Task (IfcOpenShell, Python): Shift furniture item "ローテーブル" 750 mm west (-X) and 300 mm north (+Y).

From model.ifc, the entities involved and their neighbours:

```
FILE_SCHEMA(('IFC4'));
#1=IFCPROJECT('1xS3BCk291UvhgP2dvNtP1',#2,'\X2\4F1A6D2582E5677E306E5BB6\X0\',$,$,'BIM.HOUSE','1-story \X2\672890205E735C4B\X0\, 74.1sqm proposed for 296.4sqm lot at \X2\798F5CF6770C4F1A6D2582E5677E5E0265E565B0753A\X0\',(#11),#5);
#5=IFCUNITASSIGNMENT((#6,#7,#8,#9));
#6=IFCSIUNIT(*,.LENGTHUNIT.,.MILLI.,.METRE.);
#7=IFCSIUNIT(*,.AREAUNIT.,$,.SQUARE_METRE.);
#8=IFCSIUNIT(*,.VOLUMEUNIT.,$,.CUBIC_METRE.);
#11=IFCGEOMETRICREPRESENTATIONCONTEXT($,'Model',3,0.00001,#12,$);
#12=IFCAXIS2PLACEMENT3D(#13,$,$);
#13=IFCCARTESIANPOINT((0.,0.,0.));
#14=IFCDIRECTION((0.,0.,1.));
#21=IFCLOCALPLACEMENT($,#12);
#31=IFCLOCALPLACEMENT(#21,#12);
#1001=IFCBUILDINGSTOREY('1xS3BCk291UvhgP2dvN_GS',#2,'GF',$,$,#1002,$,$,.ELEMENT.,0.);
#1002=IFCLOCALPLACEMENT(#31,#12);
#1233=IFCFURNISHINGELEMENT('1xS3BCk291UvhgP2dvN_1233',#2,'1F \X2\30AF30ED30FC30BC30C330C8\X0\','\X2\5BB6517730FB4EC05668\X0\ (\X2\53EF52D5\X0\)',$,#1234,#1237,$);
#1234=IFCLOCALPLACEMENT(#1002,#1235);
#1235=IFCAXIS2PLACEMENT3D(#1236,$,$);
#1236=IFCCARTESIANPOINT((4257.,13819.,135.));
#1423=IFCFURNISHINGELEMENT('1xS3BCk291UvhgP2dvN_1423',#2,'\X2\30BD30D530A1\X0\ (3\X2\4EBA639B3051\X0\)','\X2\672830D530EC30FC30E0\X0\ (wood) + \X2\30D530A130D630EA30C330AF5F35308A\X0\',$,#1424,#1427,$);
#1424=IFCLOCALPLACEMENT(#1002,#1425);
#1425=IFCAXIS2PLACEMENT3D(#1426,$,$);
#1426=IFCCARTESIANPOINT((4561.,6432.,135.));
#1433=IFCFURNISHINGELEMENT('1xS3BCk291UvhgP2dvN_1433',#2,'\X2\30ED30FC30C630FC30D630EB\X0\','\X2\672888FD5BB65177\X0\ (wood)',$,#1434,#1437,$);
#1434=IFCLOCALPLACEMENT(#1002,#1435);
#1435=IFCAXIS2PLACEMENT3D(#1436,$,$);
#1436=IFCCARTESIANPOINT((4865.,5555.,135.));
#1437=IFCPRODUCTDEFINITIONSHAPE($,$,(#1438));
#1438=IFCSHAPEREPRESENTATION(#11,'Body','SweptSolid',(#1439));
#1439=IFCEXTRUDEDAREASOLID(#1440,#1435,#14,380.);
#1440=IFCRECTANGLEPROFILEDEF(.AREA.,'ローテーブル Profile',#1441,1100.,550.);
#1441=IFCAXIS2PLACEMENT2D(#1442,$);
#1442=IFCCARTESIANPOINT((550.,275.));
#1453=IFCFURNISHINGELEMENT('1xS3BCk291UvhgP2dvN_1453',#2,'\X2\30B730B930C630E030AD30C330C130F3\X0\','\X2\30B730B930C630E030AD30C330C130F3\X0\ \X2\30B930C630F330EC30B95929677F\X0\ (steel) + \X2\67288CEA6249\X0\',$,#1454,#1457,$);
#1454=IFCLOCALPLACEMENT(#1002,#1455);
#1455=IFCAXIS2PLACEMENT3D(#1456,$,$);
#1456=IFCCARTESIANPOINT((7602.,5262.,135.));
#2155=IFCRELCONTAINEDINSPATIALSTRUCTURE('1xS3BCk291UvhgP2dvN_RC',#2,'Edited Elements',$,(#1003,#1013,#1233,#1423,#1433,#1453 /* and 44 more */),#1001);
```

```python
import ifcopenshell
import ifcopenshell.api.geometry
import ifcopenshell.util.placement
import ifcopenshell.util.unit

model = ifcopenshell.open("model.ifc")
unit_scale = ifcopenshell.util.unit.calculate_unit_scale(model)

item = model.by_guid("1xS3BCk291UvhgP2dvN_1433")
matrix = ifcopenshell.util.placement.get_local_placement(item.ObjectPlacement)
matrix[0, 3] -= 0.75 / unit_scale
matrix[1, 3] += 0.3 / unit_scale
ifcopenshell.api.geometry.edit_object_placement(model, product=item, matrix=matrix, is_si=False)

print(ifcopenshell.util.placement.get_local_placement(item.ObjectPlacement).round(3) + 0.0)

model.write("model_edited.ifc")
```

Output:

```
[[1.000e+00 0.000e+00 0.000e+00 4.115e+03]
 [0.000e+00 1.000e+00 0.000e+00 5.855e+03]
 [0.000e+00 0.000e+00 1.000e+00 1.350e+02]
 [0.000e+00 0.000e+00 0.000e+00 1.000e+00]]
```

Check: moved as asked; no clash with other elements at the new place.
